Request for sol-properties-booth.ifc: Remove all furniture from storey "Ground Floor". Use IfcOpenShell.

First a look at what the model holds.

```python
import ifcopenshell
import ifcopenshell.util.element

model = ifcopenshell.open("sol-properties-booth.ifc")
print(model.schema)
storey = next(s for s in model.by_type("IfcBuildingStorey") if s.Name == "Ground Floor")
furniture = [e for e in ifcopenshell.util.element.get_decomposition(storey) if e.is_a("IfcFurnishingElement")]
seen = {}
for e in furniture:
    element_type = ifcopenshell.util.element.get_type(e)
    name = element_type.Name if element_type not in (None, e) else None
    seen[name] = seen.get(name, 0) + 1
for name, count in sorted(seen.items(), key=str):
    print(count, "x", name)
```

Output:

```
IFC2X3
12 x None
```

```python
import ifcopenshell
import ifcopenshell.api.root
import ifcopenshell.util.element

model = ifcopenshell.open("sol-properties-booth.ifc")

storey = next(s for s in model.by_type("IfcBuildingStorey") if s.Name == "Ground Floor")
furniture = [e for e in ifcopenshell.util.element.get_decomposition(storey) if e.is_a("IfcFurnishingElement")]

for e in furniture:
    ifcopenshell.api.root.remove_product(model, product=e)
print(len(furniture), "removed")

model.write("sol-properties-booth-out.ifc")
```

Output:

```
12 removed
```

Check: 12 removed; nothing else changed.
